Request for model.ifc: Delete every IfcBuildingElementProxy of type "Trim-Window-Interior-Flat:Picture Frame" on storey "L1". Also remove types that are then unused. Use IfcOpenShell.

First a look at what the model holds.

```python
import ifcopenshell
import ifcopenshell.util.element

model = ifcopenshell.open("model.ifc")
print(model.schema)
storey = next(s for s in model.by_type("IfcBuildingStorey") if s.Name == "L1")
proxies = [e for e in ifcopenshell.util.element.get_decomposition(storey) if e.is_a("IfcBuildingElementProxy")]
seen = {}
for e in proxies:
    element_type = ifcopenshell.util.element.get_type(e)
    name = element_type.Name if element_type not in (None, e) else None
    seen[name] = seen.get(name, 0) + 1
for name, count in sorted(seen.items(), key=str):
    print(count, "x", name)
```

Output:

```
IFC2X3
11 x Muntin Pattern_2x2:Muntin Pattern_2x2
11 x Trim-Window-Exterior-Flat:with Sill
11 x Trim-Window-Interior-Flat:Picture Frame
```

```python
import ifcopenshell
import ifcopenshell.api.root
import ifcopenshell.util.element

model = ifcopenshell.open("model.ifc")

storey = next(s for s in model.by_type("IfcBuildingStorey") if s.Name == "L1")
proxies = [e for e in ifcopenshell.util.element.get_decomposition(storey) if e.is_a("IfcBuildingElementProxy")]
targets = [e for e in proxies if (t := ifcopenshell.util.element.get_type(e)) not in (None, e) and t.Name == "Trim-Window-Interior-Flat:Picture Frame"]
types = {ifcopenshell.util.element.get_type(e) for e in targets} - {None, *targets}

for e in targets:
    ifcopenshell.api.root.remove_product(model, product=e)
print(len(targets), "removed")

unused = [t for t in types if not ifcopenshell.util.element.get_types(t)]
for t in unused:
    ifcopenshell.api.root.remove_product(model, product=t)
print(len(unused), "unused types removed")

model.write("model_updated.ifc")
```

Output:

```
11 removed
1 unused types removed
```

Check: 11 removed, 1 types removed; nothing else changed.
